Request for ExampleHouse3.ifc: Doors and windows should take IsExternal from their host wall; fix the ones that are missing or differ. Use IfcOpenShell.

First a look at what the model holds.

```python
import ifcopenshell
import ifcopenshell.util.element

model = ifcopenshell.open("ExampleHouse3.ifc")
print(model.schema)
seen = {}
for e in model.by_type("IfcDoor") + model.by_type("IfcWindow"):
    if not e.FillsVoids:
        continue
    host = e.FillsVoids[0].RelatingOpeningElement.VoidsElements[0].RelatingBuildingElement
    own = ifcopenshell.util.element.get_pset(e, f"Pset_{e.is_a()[3:].removesuffix('StandardCase')}Common", "IsExternal")
    wall = ifcopenshell.util.element.get_pset(host, "Pset_WallCommon", "IsExternal")
    seen[e.is_a(), own, wall] = seen.get((e.is_a(), own, wall), 0) + 1
for (cls, own, wall), count in sorted(seen.items(), key=str):
    print(count, cls, "IsExternal:", own, "| host wall:", wall)
```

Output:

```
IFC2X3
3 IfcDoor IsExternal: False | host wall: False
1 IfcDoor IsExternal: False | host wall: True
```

```python
import ifcopenshell
import ifcopenshell.api.pset
import ifcopenshell.util.element

model = ifcopenshell.open("ExampleHouse3.ifc")

count = 0
for ifc_class, pset_name in (("IfcDoor", "Pset_DoorCommon"), ("IfcWindow", "Pset_WindowCommon")):
    for e in model.by_type(ifc_class):
        if not e.FillsVoids:
            continue
        host = e.FillsVoids[0].RelatingOpeningElement.VoidsElements[0].RelatingBuildingElement
        external = ifcopenshell.util.element.get_pset(host, "Pset_WallCommon", "IsExternal")
        if external is None or ifcopenshell.util.element.get_pset(e, pset_name, "IsExternal") == external:
            continue
        pset = ifcopenshell.api.pset.add_pset(model, product=e, name=pset_name)
        ifcopenshell.api.pset.edit_pset(model, pset=pset, properties={"IsExternal": external})
        count += 1

print(count, "updated")

model.write("ExampleHouse3_rev.ifc")
```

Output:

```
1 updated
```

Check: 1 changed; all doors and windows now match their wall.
